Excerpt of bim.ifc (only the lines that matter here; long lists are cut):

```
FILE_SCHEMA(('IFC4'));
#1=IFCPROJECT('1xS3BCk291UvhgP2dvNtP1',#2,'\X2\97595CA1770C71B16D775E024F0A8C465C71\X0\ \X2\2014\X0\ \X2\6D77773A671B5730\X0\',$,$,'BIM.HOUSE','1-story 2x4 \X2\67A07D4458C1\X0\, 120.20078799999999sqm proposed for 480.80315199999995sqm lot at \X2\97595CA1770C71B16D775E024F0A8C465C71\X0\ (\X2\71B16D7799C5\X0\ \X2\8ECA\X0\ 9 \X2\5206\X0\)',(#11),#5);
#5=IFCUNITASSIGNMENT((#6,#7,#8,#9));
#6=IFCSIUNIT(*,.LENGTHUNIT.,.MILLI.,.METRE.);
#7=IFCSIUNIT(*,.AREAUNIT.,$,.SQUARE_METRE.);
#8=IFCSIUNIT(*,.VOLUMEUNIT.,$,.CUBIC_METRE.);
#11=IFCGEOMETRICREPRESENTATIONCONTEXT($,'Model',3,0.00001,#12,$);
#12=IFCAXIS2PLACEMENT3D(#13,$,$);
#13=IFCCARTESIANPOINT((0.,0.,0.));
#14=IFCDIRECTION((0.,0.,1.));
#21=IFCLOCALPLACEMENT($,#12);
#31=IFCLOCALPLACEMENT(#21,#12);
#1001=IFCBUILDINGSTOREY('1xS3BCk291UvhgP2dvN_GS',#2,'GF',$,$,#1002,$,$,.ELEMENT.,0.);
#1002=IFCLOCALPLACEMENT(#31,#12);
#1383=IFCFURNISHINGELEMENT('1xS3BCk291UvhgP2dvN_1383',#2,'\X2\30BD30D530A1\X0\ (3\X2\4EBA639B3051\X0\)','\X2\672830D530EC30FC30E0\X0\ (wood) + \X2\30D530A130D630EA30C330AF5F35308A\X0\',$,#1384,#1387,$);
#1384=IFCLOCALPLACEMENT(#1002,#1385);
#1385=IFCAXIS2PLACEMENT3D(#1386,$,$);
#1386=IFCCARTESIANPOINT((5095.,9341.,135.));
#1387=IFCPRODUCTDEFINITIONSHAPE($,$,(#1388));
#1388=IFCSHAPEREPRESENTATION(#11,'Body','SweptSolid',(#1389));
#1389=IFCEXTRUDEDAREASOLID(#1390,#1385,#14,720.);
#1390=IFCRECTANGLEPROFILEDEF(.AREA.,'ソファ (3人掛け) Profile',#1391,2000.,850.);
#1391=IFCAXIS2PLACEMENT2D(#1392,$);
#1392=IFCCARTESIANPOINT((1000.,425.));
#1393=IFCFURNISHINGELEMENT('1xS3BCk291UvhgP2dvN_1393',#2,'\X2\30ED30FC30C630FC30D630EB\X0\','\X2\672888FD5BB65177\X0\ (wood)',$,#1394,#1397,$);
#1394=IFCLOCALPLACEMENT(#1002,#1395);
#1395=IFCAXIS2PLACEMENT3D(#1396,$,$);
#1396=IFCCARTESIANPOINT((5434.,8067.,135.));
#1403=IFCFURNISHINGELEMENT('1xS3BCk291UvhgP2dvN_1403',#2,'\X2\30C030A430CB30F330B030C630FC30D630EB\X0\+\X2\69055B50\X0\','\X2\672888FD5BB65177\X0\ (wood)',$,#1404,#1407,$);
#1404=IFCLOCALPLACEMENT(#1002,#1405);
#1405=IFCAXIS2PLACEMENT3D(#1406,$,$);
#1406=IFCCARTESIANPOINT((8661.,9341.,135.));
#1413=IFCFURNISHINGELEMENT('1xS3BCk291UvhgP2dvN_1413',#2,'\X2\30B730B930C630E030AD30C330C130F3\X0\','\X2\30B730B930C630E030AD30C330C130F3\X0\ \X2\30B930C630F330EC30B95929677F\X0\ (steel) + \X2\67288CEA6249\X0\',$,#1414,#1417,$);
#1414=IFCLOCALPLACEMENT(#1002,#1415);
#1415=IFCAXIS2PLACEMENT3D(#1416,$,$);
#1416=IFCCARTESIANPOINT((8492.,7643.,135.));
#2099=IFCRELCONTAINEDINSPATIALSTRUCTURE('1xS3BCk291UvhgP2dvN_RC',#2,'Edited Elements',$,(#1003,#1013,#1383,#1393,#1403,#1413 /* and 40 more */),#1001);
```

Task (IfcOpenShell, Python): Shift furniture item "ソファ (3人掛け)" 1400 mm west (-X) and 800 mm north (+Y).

```python
import ifcopenshell
import ifcopenshell.api.geometry
import ifcopenshell.util.placement
import ifcopenshell.util.unit

model = ifcopenshell.open("bim.ifc")
unit_scale = ifcopenshell.util.unit.calculate_unit_scale(model)

item = model.by_guid("1xS3BCk291UvhgP2dvN_1383")
matrix = ifcopenshell.util.placement.get_local_placement(item.ObjectPlacement)
matrix[0, 3] -= 1.4 / unit_scale
matrix[1, 3] += 0.8 / unit_scale
ifcopenshell.api.geometry.edit_object_placement(model, product=item, matrix=matrix, is_si=False)

print(ifcopenshell.util.placement.get_local_placement(item.ObjectPlacement).round(3) + 0.0)

model.write("bim_edited.ifc")
```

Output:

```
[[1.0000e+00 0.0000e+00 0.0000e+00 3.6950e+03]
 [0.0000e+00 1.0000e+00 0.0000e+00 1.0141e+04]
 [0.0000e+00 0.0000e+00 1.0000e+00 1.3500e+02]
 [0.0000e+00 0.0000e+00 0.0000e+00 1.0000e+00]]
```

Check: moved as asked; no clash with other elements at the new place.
